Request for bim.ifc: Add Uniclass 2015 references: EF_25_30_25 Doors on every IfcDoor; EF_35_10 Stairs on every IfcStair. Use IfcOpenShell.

First a look at what the model holds.

```python
import ifcopenshell

model = ifcopenshell.open("bim.ifc")
print(model.schema)
print("classifications:", [c.Name for c in model.by_type("IfcClassification")])
for ifc_class in ("IfcDoor", "IfcRoof", "IfcStair", "IfcWall", "IfcWindow"):
    print(ifc_class, len(model.by_type(ifc_class)))
```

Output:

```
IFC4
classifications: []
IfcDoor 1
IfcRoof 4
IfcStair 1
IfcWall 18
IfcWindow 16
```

```python
import ifcopenshell
import ifcopenshell.api.classification

model = ifcopenshell.open("bim.ifc")

system = ifcopenshell.api.classification.add_classification(model, classification="Uniclass 2015")

codes = {
    "IfcDoor": ("EF_25_30_25", "Doors"),
    "IfcStair": ("EF_35_10", "Stairs"),
}
for ifc_class, (code, name) in codes.items():
    products = model.by_type(ifc_class)
    ifcopenshell.api.classification.add_reference(
        model, products=products, classification=system, identification=code, name=name
    )
    print(code, len(products))

model.write("bim_edited.ifc")
```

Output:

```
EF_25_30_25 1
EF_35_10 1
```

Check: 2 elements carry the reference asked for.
